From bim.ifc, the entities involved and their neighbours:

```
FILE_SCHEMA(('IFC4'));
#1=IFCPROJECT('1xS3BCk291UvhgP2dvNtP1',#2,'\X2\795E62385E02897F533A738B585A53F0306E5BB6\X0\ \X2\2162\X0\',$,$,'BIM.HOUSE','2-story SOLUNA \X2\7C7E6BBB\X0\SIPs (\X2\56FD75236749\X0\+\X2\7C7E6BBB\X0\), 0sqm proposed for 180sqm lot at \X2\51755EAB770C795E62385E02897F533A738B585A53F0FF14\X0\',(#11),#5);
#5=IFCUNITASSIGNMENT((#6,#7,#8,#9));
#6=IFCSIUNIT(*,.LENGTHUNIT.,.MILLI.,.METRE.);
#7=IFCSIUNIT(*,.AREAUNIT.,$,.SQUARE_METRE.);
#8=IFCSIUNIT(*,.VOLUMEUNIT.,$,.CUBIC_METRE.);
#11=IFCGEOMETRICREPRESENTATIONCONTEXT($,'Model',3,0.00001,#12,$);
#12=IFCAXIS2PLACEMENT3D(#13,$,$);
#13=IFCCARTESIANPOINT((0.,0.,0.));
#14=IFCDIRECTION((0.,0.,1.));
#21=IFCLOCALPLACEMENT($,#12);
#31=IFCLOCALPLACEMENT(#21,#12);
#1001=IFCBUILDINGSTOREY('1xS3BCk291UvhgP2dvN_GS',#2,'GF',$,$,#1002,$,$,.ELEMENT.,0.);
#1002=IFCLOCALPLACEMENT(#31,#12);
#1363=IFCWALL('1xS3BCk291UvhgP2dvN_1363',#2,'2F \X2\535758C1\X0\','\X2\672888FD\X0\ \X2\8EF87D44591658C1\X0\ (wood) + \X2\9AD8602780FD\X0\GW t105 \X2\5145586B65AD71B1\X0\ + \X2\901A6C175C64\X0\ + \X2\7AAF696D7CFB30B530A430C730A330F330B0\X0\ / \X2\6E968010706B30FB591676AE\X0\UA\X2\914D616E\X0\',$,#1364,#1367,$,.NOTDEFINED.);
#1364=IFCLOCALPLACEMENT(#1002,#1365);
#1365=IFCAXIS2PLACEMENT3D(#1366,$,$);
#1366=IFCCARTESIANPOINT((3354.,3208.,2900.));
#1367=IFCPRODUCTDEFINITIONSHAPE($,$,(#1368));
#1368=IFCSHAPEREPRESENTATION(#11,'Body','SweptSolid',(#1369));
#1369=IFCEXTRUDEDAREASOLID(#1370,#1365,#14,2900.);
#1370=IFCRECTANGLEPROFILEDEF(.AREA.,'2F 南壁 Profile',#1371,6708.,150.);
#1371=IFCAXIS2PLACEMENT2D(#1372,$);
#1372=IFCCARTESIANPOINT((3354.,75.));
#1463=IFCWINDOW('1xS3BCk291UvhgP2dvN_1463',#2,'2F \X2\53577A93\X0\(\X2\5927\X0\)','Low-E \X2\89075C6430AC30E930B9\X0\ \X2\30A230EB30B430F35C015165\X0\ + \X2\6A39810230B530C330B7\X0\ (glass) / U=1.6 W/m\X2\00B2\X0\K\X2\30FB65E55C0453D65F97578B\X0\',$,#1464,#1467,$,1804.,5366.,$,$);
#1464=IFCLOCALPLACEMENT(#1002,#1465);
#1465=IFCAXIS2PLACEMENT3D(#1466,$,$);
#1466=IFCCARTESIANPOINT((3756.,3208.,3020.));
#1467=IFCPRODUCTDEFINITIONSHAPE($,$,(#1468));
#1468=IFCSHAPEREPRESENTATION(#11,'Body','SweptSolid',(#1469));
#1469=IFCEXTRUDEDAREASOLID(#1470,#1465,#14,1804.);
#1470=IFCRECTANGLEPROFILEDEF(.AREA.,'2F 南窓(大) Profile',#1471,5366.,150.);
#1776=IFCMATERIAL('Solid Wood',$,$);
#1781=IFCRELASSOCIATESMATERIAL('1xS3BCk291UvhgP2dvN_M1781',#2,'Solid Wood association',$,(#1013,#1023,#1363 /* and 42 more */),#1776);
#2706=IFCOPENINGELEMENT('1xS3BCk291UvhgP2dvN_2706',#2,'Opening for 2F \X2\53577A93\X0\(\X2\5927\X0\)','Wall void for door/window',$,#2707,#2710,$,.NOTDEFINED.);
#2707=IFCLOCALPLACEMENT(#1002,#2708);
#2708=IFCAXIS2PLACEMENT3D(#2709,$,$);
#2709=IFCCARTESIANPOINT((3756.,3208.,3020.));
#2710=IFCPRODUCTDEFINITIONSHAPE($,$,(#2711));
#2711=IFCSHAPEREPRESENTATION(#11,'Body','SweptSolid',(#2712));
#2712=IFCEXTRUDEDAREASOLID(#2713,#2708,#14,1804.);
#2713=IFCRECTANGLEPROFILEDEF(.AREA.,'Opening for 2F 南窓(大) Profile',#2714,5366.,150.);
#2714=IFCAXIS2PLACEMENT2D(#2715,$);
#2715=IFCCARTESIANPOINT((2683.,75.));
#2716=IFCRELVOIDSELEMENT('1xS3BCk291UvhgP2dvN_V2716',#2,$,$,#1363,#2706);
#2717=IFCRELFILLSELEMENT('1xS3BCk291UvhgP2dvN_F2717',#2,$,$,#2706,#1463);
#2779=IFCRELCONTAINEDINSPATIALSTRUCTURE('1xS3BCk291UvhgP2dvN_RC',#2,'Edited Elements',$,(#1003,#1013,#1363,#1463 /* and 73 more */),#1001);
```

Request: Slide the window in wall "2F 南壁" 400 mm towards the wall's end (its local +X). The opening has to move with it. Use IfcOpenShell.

```python
import ifcopenshell
import ifcopenshell.api.geometry
import ifcopenshell.util.placement

model = ifcopenshell.open("bim.ifc")

window = model.by_guid("1xS3BCk291UvhgP2dvN_1463")
opening = window.FillsVoids[0].RelatingOpeningElement
wall = opening.VoidsElements[0].RelatingBuildingElement

wall_matrix = ifcopenshell.util.placement.get_local_placement(wall.ObjectPlacement)
shift = wall_matrix[:3, 0] * 400.0
before = ifcopenshell.util.placement.get_local_placement(window.ObjectPlacement)[:3, 3].copy()

# The window is not placed relative to its opening, so move both.
for product in (opening, window):
    matrix = ifcopenshell.util.placement.get_local_placement(product.ObjectPlacement)
    matrix[:3, 3] += shift
    ifcopenshell.api.geometry.edit_object_placement(model, product=product, matrix=matrix, is_si=False)

after = ifcopenshell.util.placement.get_local_placement(window.ObjectPlacement)[:3, 3]
print("window moved by", (after - before).round(3) + 0.0)

model.write("bim_edited.ifc")
```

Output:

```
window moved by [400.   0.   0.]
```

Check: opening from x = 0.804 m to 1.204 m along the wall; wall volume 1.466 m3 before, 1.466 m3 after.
